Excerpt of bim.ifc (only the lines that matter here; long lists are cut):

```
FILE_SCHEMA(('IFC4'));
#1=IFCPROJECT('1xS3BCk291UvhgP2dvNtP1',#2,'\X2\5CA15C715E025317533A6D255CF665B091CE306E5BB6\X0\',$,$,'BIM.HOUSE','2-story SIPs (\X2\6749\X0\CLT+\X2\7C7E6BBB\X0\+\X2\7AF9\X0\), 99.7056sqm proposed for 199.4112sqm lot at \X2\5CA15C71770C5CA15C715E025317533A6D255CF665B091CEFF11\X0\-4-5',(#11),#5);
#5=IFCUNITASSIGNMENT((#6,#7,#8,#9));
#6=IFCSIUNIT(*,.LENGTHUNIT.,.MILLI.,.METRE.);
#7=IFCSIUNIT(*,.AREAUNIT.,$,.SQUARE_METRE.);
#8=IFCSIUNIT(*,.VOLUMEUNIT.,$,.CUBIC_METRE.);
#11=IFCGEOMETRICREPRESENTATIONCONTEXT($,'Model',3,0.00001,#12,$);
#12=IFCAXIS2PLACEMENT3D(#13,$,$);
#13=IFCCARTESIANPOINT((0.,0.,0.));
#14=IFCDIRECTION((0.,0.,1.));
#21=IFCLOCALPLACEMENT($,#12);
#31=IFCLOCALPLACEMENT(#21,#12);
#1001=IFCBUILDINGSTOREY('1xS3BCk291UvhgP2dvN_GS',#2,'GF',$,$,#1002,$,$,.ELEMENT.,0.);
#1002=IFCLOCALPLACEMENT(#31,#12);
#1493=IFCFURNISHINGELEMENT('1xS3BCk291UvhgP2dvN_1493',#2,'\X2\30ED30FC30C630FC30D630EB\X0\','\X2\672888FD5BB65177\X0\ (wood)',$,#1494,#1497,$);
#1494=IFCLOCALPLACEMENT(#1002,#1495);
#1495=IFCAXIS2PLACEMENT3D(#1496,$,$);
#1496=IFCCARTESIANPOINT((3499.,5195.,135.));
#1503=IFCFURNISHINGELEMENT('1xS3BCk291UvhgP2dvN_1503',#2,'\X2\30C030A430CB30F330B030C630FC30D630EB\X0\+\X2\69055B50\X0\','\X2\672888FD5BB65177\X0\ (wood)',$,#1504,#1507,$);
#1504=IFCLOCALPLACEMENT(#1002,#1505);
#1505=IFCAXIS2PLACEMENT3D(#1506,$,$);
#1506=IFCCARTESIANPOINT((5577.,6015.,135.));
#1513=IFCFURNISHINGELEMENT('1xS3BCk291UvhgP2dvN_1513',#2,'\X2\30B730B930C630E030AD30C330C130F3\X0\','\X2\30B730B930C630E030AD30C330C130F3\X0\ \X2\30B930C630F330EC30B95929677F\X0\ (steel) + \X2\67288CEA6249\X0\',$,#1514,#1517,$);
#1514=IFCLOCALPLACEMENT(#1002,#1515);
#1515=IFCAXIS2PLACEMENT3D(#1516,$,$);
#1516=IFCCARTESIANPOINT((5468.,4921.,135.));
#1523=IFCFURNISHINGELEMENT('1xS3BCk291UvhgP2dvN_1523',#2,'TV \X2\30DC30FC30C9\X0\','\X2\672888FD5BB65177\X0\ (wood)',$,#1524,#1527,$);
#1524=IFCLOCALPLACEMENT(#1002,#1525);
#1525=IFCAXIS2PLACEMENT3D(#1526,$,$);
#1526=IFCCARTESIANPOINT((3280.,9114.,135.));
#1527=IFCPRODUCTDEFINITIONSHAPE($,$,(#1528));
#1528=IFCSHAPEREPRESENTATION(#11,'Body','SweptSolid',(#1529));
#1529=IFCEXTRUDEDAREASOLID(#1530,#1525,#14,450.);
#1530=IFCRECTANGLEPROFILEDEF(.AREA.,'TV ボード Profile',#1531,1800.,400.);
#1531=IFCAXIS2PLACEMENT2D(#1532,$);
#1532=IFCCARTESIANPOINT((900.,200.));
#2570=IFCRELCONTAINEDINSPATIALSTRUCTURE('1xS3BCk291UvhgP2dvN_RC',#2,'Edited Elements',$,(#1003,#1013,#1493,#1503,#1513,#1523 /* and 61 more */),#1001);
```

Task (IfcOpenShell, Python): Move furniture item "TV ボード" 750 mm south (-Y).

```python
import ifcopenshell
import ifcopenshell.api.geometry
import ifcopenshell.util.placement
import ifcopenshell.util.unit

model = ifcopenshell.open("bim.ifc")
unit_scale = ifcopenshell.util.unit.calculate_unit_scale(model)

item = model.by_id(1523)
matrix = ifcopenshell.util.placement.get_local_placement(item.ObjectPlacement)
matrix[1, 3] -= 0.75 / unit_scale
ifcopenshell.api.geometry.edit_object_placement(model, product=item, matrix=matrix, is_si=False)

print(ifcopenshell.util.placement.get_local_placement(item.ObjectPlacement).round(3) + 0.0)

model.write("bim-out.ifc")
```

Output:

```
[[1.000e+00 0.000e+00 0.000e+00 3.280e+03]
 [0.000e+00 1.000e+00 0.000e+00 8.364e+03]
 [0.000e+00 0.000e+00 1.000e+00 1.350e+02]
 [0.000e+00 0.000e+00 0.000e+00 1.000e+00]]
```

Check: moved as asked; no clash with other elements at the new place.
